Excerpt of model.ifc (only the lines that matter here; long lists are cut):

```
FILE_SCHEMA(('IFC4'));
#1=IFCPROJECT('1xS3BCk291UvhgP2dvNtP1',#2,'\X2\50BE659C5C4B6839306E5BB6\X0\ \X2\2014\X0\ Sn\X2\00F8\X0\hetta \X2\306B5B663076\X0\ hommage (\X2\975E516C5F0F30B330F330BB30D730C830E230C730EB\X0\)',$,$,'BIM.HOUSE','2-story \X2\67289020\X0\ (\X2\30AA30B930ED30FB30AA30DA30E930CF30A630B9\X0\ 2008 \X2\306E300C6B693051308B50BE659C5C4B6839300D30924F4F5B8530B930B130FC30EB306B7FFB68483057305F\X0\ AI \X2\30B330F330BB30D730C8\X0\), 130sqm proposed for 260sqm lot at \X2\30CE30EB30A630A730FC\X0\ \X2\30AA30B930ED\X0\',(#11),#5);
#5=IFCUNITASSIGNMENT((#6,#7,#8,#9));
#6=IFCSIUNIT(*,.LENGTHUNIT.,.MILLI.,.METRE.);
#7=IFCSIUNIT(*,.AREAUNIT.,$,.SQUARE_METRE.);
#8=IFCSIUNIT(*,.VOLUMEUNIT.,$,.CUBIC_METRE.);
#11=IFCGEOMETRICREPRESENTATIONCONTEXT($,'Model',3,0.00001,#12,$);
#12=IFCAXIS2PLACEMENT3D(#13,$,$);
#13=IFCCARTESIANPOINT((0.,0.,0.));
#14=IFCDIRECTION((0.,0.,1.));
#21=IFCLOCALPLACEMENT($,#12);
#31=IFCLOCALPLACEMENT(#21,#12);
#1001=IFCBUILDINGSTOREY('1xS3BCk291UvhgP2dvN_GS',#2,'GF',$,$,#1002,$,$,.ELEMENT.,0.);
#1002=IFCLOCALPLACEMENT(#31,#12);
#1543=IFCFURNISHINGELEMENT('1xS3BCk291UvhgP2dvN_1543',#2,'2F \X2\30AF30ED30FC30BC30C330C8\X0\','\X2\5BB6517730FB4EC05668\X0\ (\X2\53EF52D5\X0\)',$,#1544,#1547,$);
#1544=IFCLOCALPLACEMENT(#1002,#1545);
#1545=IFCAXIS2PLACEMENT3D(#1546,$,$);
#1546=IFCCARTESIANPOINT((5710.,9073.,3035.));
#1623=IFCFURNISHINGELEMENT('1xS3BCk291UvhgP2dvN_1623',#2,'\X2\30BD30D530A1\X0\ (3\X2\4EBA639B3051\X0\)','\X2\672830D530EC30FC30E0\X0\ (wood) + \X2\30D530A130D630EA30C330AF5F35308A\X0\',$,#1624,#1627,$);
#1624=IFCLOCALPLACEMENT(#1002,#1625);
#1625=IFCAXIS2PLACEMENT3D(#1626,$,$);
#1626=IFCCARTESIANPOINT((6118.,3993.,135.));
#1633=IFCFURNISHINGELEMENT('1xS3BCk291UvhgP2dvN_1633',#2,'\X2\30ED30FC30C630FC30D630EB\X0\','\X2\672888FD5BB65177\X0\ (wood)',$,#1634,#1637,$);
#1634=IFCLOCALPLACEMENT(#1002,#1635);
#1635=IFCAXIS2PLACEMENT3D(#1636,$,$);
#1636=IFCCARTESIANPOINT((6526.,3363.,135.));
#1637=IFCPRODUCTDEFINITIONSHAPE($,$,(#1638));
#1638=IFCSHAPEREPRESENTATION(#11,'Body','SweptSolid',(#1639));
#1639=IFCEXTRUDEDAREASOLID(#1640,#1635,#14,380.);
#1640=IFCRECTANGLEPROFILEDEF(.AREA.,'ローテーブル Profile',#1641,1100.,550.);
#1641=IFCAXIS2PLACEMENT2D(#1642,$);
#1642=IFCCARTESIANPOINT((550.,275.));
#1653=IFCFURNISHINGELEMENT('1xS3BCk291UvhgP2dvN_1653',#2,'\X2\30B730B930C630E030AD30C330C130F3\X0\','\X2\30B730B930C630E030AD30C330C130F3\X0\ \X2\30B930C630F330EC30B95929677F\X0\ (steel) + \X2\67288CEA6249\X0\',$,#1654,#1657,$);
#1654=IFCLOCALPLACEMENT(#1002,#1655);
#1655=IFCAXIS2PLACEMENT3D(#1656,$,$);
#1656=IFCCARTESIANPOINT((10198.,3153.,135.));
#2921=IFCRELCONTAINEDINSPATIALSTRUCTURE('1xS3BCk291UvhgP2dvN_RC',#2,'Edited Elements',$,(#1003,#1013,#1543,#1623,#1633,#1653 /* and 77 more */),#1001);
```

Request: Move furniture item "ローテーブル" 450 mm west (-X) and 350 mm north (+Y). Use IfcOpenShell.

```python
import ifcopenshell
import ifcopenshell.api.geometry
import ifcopenshell.util.placement

model = ifcopenshell.open("model.ifc")

item = model.by_id(1633)
matrix = ifcopenshell.util.placement.get_local_placement(item.ObjectPlacement)
matrix[0, 3] -= 450.0
matrix[1, 3] += 350.0
ifcopenshell.api.geometry.edit_object_placement(model, product=item, matrix=matrix, is_si=False)

print(ifcopenshell.util.placement.get_local_placement(item.ObjectPlacement).round(3) + 0.0)

model.write("model_v2.ifc")
```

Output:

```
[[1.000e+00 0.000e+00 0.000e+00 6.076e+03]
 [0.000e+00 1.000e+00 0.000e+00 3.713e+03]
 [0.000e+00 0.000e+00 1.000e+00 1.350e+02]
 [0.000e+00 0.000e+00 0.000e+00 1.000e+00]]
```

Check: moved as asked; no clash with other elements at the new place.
